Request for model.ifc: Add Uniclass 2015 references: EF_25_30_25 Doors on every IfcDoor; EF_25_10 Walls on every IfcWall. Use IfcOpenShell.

First a look at what the model holds.

```python
import ifcopenshell

model = ifcopenshell.open("model.ifc")
print(model.schema)
print("classifications:", [c.Name for c in model.by_type("IfcClassification")])
for ifc_class in ("IfcDoor", "IfcRoof", "IfcStair", "IfcWall", "IfcWindow"):
    print(ifc_class, len(model.by_type(ifc_class)))
```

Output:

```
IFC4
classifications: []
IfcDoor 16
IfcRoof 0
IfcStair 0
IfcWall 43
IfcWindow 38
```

```python
import ifcopenshell
import ifcopenshell.api.classification

model = ifcopenshell.open("model.ifc")

system = ifcopenshell.api.classification.add_classification(model, classification="Uniclass 2015")

codes = {
    "IfcDoor": ("EF_25_30_25", "Doors"),
    "IfcWall": ("EF_25_10", "Walls"),
}
for ifc_class, (code, name) in codes.items():
    products = model.by_type(ifc_class)
    ifcopenshell.api.classification.add_reference(
        model, products=products, classification=system, identification=code, name=name
    )
    print(code, len(products))

model.write("model_edited.ifc")
```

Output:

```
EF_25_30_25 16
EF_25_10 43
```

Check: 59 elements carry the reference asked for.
